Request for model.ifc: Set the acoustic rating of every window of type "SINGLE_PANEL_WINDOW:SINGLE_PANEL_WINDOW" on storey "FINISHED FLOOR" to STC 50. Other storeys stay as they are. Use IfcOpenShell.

First a look at what the model holds.

```python
import ifcopenshell
import ifcopenshell.util.element

model = ifcopenshell.open("model.ifc")
print(model.schema)
storey = next(s for s in model.by_type("IfcBuildingStorey") if s.Name == "FINISHED FLOOR")
windows = [e for e in ifcopenshell.util.element.get_decomposition(storey) if e.is_a("IfcWindow")]
seen = {}
for e in windows:
    element_type = ifcopenshell.util.element.get_type(e)
    key = (element_type.Name if element_type != e and element_type else None, ifcopenshell.util.element.get_pset(e, "Pset_WindowCommon", "AcousticRating"))
    seen[key] = seen.get(key, 0) + 1
for (name, value), count in sorted(seen.items(), key=str):
    print(count, "x", name, "|", value)
```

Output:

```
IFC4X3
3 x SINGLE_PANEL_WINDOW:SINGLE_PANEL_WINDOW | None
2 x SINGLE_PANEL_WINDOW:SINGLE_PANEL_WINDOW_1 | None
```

```python
import ifcopenshell
import ifcopenshell.api.pset
import ifcopenshell.util.element

model = ifcopenshell.open("model.ifc")

storey = next(s for s in model.by_type("IfcBuildingStorey") if s.Name == "FINISHED FLOOR")
windows = [e for e in ifcopenshell.util.element.get_decomposition(storey) if e.is_a("IfcWindow")]

count = 0
for e in windows:
    element_type = ifcopenshell.util.element.get_type(e)
    if element_type in (None, e) or element_type.Name != "SINGLE_PANEL_WINDOW:SINGLE_PANEL_WINDOW":
        continue
    # add_pset returns the element's existing set when there is one.
    pset = ifcopenshell.api.pset.add_pset(model, product=e, name="Pset_WindowCommon")
    ifcopenshell.api.pset.edit_pset(model, pset=pset, properties={"AcousticRating": "STC 50"})
    count += 1

print(count, "windows updated")

model.write("model_rev.ifc")
```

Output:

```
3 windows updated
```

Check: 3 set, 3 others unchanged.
